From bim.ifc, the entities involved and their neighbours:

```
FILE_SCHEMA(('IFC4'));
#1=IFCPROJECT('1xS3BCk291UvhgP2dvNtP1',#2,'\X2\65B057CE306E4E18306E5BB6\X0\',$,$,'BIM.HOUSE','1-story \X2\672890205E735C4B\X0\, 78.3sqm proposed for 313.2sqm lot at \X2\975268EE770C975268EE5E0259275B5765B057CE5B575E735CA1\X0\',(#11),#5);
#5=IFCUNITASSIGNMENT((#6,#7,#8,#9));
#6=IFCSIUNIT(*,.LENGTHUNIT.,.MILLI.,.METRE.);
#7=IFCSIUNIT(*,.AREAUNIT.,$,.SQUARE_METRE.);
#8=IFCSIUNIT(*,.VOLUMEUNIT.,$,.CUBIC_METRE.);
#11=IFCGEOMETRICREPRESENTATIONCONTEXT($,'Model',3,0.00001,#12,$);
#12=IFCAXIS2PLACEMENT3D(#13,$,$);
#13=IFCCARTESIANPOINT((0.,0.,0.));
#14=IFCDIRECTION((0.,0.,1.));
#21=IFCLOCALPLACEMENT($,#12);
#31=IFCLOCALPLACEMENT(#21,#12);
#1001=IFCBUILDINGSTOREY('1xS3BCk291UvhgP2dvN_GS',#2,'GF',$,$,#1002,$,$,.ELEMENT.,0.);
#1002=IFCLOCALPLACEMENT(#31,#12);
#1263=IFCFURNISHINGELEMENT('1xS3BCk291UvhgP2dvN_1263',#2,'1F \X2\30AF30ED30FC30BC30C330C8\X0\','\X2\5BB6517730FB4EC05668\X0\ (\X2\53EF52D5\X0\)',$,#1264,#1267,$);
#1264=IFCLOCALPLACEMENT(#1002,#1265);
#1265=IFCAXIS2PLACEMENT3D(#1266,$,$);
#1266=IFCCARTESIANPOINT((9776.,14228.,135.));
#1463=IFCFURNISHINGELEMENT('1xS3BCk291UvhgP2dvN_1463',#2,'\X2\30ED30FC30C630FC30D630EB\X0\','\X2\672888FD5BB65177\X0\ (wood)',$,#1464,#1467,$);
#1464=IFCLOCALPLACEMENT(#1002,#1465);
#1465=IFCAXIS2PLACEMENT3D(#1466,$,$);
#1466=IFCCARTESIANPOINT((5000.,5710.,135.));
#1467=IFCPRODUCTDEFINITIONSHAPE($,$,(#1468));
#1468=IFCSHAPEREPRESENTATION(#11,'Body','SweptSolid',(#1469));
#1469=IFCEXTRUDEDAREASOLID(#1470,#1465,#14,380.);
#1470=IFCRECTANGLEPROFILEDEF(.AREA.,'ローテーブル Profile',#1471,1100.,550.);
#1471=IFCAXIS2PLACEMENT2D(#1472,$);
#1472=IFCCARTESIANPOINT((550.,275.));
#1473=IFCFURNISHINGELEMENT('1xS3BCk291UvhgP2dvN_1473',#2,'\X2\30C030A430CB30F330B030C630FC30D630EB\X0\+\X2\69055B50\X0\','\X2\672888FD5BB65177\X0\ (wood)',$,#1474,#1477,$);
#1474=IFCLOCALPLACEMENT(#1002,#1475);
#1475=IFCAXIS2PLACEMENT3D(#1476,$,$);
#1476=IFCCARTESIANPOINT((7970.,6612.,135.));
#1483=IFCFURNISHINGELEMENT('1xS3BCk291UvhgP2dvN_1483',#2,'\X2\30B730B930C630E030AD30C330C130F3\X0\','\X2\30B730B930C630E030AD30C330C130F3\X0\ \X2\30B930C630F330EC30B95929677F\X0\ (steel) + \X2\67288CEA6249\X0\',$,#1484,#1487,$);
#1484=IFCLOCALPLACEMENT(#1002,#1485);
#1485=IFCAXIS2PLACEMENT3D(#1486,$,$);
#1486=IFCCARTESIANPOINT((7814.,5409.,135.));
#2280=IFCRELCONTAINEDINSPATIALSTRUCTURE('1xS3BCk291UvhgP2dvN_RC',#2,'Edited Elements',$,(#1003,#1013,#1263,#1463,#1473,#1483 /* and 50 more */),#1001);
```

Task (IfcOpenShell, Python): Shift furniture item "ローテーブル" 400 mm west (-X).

```python
import ifcopenshell
import ifcopenshell.api.geometry
import ifcopenshell.util.placement

model = ifcopenshell.open("bim.ifc")

item = model.by_guid("1xS3BCk291UvhgP2dvN_1463")
matrix = ifcopenshell.util.placement.get_local_placement(item.ObjectPlacement)
matrix[0, 3] -= 400.0
ifcopenshell.api.geometry.edit_object_placement(model, product=item, matrix=matrix, is_si=False)

print(ifcopenshell.util.placement.get_local_placement(item.ObjectPlacement).round(3) + 0.0)

model.write("bim_edited.ifc")
```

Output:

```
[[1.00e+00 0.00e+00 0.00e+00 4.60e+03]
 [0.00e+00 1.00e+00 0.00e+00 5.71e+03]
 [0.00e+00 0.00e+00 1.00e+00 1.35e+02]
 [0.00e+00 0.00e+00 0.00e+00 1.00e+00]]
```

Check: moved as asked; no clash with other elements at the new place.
